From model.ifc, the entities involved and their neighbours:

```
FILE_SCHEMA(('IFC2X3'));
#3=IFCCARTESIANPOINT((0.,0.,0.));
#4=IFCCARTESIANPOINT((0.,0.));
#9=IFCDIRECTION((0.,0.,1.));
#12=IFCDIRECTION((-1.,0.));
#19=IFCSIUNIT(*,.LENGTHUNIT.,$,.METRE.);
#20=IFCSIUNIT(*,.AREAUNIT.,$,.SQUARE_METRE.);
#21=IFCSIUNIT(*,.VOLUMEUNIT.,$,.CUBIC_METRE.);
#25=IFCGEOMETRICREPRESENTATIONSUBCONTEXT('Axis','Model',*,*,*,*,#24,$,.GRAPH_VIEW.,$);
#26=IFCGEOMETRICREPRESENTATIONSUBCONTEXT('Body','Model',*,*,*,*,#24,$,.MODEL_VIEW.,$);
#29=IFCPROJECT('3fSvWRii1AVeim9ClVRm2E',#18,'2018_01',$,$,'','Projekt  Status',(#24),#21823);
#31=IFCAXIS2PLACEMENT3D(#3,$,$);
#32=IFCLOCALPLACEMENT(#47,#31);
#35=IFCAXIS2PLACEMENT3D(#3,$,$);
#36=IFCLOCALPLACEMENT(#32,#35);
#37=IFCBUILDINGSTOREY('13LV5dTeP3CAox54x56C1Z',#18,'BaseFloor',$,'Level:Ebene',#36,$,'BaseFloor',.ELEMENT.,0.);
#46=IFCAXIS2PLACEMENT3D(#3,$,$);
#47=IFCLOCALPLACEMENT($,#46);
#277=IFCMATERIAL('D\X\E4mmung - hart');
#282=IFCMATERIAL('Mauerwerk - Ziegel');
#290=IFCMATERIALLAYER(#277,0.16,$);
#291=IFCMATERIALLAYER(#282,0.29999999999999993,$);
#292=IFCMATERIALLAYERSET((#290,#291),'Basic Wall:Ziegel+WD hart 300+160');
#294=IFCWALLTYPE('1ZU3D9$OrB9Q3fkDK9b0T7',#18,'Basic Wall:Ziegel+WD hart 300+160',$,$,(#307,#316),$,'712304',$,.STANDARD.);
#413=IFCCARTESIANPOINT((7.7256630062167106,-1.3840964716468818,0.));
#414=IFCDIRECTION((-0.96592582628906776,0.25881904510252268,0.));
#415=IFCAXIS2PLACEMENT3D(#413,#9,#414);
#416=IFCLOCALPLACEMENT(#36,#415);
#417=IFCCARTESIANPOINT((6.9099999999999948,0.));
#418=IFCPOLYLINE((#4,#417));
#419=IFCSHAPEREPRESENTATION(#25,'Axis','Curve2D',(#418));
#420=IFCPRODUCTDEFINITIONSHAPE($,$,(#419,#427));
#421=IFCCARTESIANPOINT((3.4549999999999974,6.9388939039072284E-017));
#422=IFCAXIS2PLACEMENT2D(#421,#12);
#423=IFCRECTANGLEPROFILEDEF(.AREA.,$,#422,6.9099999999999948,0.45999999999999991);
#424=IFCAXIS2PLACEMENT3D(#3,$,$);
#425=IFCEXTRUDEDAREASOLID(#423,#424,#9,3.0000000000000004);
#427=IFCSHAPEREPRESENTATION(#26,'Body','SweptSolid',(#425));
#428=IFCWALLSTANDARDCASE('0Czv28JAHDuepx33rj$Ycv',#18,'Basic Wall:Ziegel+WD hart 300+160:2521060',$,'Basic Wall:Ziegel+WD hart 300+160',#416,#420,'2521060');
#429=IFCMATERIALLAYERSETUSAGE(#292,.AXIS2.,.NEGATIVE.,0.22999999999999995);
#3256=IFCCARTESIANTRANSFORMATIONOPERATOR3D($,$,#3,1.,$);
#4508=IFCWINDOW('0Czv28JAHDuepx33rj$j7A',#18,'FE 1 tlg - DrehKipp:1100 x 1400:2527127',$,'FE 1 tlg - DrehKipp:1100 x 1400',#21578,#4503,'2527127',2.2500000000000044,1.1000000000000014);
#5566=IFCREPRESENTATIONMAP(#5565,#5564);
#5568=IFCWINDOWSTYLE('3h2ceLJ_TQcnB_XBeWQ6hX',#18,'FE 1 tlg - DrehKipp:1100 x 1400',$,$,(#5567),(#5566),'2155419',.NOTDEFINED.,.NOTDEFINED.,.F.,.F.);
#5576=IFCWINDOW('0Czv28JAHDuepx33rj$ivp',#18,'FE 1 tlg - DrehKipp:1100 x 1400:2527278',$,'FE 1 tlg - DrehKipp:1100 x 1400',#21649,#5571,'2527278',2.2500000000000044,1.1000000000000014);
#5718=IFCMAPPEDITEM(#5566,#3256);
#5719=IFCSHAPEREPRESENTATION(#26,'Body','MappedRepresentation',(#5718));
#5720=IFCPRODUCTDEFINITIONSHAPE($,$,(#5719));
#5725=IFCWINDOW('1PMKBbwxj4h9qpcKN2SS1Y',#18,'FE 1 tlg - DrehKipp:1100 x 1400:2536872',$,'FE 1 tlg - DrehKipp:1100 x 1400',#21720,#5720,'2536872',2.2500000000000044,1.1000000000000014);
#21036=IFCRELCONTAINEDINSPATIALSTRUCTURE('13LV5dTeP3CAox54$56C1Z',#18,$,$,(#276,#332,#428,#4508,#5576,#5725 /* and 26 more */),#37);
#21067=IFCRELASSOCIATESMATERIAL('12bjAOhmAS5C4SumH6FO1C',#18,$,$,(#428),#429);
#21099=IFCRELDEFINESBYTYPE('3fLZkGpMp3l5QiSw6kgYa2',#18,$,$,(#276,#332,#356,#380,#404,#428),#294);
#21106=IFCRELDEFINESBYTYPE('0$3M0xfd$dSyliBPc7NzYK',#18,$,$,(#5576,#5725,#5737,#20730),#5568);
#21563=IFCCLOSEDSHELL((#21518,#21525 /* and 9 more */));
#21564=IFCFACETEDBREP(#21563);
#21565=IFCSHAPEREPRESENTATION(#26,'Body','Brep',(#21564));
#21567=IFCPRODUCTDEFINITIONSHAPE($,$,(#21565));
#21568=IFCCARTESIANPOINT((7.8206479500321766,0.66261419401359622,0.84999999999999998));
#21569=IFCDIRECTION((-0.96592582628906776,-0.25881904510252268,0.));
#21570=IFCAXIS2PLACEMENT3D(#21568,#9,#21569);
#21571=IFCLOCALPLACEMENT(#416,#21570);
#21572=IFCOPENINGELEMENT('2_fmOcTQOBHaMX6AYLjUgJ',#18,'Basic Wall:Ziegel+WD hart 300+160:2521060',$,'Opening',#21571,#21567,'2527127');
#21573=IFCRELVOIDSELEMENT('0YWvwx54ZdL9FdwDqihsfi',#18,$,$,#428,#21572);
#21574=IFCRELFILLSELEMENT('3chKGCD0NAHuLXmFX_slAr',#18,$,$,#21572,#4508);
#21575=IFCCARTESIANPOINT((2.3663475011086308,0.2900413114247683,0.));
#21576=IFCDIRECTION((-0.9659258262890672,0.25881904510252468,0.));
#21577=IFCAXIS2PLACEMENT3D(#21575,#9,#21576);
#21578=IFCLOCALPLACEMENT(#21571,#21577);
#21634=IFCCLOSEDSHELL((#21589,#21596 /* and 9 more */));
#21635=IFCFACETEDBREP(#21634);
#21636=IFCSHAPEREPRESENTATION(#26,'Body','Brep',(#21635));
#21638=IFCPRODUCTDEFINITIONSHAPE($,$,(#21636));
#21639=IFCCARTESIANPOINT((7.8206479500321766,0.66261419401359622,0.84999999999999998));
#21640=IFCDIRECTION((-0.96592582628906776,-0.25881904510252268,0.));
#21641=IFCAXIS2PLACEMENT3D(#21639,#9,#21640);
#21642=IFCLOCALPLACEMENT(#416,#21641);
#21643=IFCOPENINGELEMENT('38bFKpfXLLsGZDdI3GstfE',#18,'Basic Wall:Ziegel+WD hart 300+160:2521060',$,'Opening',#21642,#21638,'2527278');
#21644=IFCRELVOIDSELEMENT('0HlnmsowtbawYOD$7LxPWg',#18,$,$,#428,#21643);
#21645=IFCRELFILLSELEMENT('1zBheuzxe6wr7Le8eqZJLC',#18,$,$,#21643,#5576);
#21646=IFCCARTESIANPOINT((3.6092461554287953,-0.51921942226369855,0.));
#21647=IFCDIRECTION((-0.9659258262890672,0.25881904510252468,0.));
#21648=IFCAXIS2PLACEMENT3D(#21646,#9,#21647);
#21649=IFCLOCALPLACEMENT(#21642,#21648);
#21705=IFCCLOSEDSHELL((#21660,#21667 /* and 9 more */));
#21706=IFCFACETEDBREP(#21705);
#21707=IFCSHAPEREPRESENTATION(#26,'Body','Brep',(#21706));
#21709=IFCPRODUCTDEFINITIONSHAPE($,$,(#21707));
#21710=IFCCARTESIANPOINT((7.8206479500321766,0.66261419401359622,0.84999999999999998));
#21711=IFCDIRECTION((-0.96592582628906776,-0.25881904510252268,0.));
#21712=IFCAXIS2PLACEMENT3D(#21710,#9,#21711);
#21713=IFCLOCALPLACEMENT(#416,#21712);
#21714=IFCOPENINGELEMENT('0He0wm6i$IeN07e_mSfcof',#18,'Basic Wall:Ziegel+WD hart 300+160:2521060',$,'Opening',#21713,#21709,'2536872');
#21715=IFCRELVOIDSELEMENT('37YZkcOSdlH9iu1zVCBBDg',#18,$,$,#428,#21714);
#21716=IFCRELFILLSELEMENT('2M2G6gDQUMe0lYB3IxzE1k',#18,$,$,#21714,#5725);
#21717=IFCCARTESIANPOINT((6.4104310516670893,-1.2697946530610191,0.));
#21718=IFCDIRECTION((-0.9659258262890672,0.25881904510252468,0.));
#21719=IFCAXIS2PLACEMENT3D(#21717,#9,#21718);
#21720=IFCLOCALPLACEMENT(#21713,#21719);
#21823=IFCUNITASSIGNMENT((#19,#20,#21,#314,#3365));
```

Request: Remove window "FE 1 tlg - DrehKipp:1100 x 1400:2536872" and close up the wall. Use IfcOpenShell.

```python
import ifcopenshell
import ifcopenshell.api.feature
import ifcopenshell.api.root
import ifcopenshell.geom
import ifcopenshell.util.shape

model = ifcopenshell.open("model.ifc")
settings = ifcopenshell.geom.settings()


def volume(element):
    """Net volume in cubic metres, openings subtracted."""
    shape = ifcopenshell.geom.create_shape(settings, element)
    return ifcopenshell.util.shape.get_volume(shape.geometry)


window = model.by_guid("1PMKBbwxj4h9qpcKN2SS1Y")
opening = window.FillsVoids[0].RelatingOpeningElement
wall = opening.VoidsElements[0].RelatingBuildingElement
before = volume(wall)

ifcopenshell.api.root.remove_product(model, product=window)
ifcopenshell.api.feature.remove_feature(model, feature=opening)

after = volume(wall)

print(f"wall volume {before:.3f} -> {after:.3f} m3")

model.write("model_rev.ifc")
```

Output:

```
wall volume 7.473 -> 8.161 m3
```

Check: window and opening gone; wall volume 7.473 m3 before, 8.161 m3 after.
